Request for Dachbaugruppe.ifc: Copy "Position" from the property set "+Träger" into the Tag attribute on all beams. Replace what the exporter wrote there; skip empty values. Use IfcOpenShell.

First a look at what the model holds.

```python
import ifcopenshell
import ifcopenshell.util.element

model = ifcopenshell.open("Dachbaugruppe.ifc")
print(model.schema)
beams = model.by_type("IfcBeam")
print(len(beams), "beams")
for e in beams[:8]:
    source = ifcopenshell.util.element.get_pset(e, "+Träger", "Position")
    target = e.Tag
    print(e.id(), repr(source), repr(target), sep=" | ")
```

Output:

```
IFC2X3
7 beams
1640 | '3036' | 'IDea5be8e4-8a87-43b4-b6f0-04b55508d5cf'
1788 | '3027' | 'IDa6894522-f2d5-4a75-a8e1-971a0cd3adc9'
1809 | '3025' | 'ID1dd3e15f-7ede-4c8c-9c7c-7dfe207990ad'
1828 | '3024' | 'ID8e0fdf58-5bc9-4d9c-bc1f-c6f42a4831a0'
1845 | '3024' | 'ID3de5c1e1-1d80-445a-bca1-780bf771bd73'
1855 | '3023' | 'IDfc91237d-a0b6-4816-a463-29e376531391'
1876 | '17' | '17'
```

```python
import ifcopenshell
import ifcopenshell.util.element

model = ifcopenshell.open("Dachbaugruppe.ifc")

count = 0
for e in model.by_type("IfcBeam"):
    value = ifcopenshell.util.element.get_pset(e, "+Träger", "Position")
    current = e.Tag
    if not value or not value.strip() or current == value:
        continue
    e.Tag = value
    count += 1

print(count, "beams updated")

model.write("Dachbaugruppe-out.ifc")
```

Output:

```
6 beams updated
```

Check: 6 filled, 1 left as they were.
